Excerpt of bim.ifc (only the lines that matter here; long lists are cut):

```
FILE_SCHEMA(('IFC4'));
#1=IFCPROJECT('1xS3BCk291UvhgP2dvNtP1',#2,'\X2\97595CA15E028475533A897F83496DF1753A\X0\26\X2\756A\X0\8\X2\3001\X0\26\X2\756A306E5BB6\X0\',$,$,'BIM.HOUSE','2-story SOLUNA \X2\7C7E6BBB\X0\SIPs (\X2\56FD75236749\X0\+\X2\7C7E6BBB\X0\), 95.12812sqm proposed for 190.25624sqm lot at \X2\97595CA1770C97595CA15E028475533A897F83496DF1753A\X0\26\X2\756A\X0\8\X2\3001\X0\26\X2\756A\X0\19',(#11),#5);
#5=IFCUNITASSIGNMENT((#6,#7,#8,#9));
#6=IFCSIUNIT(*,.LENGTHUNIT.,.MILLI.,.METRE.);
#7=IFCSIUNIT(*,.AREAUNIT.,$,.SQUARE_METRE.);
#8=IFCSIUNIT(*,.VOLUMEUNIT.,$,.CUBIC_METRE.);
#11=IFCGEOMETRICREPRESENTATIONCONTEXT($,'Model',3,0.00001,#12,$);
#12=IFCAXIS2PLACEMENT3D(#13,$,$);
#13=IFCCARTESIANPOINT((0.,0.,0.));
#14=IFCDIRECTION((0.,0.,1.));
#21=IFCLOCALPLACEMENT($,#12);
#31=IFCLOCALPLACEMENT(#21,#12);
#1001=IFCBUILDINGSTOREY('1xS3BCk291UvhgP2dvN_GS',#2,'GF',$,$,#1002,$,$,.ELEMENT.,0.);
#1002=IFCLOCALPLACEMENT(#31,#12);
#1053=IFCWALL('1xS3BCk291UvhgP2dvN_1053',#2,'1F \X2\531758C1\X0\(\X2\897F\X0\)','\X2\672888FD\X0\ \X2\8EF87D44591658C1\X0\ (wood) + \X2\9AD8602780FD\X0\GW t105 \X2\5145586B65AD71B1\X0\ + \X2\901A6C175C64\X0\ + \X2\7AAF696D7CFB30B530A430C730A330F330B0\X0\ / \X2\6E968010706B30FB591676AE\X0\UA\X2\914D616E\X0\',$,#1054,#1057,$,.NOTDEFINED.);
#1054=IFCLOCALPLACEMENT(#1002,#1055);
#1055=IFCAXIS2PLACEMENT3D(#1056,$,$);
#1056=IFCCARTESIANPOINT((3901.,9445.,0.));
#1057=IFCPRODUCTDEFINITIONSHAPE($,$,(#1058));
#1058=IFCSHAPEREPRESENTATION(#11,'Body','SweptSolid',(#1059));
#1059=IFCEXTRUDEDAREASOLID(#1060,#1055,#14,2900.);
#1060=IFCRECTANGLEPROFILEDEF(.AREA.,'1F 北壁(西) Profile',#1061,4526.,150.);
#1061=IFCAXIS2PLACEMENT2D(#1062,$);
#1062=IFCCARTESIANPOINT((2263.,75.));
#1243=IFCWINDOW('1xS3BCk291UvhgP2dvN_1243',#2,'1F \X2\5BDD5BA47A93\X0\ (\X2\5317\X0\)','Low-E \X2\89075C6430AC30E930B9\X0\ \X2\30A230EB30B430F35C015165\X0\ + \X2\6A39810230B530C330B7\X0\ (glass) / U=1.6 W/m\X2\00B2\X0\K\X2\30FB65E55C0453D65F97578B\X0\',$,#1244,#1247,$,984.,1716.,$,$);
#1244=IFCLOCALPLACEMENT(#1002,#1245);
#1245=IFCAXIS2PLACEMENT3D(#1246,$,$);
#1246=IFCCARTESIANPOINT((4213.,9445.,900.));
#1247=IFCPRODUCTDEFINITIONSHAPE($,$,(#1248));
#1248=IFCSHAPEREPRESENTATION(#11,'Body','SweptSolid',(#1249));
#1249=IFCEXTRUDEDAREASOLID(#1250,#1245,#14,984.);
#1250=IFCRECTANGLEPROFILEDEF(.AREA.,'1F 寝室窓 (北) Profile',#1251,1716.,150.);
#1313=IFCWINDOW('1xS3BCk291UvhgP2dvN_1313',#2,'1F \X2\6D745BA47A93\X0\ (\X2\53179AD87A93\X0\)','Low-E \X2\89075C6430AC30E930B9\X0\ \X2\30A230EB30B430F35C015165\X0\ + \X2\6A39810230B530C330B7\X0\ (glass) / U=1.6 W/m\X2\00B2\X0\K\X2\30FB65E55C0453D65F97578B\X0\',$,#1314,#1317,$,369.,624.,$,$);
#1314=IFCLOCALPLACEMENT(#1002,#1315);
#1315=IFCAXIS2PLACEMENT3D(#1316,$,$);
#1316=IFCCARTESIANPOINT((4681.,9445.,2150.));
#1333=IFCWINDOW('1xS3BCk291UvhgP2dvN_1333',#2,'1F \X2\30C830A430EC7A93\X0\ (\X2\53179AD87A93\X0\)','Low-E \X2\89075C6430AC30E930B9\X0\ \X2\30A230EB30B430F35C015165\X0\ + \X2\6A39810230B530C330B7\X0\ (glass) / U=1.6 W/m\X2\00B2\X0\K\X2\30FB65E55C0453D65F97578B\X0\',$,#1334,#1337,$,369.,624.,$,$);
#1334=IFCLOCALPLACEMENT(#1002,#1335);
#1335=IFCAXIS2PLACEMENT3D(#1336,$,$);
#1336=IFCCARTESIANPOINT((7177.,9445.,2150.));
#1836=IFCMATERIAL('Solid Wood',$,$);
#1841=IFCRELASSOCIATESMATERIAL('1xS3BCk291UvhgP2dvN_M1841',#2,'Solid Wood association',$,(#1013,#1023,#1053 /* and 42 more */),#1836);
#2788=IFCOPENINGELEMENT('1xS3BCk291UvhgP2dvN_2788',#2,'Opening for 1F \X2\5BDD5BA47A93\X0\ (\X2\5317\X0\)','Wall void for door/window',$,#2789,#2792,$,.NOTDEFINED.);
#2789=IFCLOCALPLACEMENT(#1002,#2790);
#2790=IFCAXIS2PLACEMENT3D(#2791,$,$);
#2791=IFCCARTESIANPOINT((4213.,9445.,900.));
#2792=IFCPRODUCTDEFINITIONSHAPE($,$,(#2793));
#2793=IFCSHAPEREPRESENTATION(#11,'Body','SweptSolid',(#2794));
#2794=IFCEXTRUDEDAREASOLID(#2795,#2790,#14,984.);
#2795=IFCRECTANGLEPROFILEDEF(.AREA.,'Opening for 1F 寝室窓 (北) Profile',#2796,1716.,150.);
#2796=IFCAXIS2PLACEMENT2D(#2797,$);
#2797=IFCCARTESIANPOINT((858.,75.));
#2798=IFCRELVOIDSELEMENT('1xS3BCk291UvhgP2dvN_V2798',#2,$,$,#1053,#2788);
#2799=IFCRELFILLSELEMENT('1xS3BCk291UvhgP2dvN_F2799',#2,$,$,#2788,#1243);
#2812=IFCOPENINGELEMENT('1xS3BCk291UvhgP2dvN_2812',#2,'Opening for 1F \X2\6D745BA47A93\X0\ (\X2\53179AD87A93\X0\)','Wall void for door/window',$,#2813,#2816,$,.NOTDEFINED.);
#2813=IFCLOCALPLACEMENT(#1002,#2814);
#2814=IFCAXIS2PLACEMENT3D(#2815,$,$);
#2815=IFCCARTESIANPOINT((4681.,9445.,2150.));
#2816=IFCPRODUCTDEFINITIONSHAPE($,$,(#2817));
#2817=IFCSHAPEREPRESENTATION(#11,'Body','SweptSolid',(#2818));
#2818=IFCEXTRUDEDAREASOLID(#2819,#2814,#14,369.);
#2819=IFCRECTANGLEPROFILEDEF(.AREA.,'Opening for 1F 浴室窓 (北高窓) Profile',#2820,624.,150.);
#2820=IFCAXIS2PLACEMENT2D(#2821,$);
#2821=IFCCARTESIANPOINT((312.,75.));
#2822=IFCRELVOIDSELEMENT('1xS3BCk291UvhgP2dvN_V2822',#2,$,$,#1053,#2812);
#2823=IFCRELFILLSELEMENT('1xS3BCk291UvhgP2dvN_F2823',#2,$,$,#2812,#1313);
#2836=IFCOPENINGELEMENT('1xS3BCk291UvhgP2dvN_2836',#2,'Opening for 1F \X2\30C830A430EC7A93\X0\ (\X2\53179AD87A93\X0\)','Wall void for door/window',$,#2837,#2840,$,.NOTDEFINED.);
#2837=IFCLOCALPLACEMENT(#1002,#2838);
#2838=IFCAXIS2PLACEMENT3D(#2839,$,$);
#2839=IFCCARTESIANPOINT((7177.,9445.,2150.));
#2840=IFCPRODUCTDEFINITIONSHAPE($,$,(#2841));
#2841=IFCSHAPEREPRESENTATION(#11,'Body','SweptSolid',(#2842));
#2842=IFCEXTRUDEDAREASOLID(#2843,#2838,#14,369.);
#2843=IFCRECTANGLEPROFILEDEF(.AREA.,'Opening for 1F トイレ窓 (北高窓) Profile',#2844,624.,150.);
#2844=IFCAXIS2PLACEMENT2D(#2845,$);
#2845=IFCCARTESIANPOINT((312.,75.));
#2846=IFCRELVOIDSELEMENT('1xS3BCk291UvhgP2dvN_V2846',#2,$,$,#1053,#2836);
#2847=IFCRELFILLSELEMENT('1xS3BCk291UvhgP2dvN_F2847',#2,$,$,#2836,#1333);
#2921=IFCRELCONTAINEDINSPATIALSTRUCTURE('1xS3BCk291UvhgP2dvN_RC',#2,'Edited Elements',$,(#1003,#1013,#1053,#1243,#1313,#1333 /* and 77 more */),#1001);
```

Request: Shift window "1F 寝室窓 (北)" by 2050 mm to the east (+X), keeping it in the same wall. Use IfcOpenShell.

```python
import ifcopenshell
import ifcopenshell.api.geometry
import ifcopenshell.util.placement
import ifcopenshell.util.unit

model = ifcopenshell.open("bim.ifc")
unit_scale = ifcopenshell.util.unit.calculate_unit_scale(model)

window = model.by_guid("1xS3BCk291UvhgP2dvN_1243")
opening = window.FillsVoids[0].RelatingOpeningElement
wall = opening.VoidsElements[0].RelatingBuildingElement

wall_matrix = ifcopenshell.util.placement.get_local_placement(wall.ObjectPlacement)
shift = wall_matrix[:3, 0] * 2.05 / unit_scale
before = ifcopenshell.util.placement.get_local_placement(window.ObjectPlacement)[:3, 3].copy()

# The window is not placed relative to its opening, so move both.
for product in (opening, window):
    matrix = ifcopenshell.util.placement.get_local_placement(product.ObjectPlacement)
    matrix[:3, 3] += shift
    ifcopenshell.api.geometry.edit_object_placement(model, product=product, matrix=matrix, is_si=False)

after = ifcopenshell.util.placement.get_local_placement(window.ObjectPlacement)[:3, 3]
print("window moved by", (after - before).round(3) + 0.0)

model.write("bim_updated.ifc")
```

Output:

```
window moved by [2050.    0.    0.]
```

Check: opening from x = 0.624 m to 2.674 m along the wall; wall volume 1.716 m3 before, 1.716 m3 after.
